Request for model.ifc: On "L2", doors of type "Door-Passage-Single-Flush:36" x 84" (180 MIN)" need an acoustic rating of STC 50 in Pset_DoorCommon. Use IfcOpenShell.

First a look at what the model holds.

```python
import ifcopenshell
import ifcopenshell.util.element

model = ifcopenshell.open("model.ifc")
print(model.schema)
storey = next(s for s in model.by_type("IfcBuildingStorey") if s.Name == "L2")
doors = [e for e in ifcopenshell.util.element.get_decomposition(storey) if e.is_a("IfcDoor")]
seen = {}
for e in doors:
    element_type = ifcopenshell.util.element.get_type(e)
    key = (element_type.Name if element_type != e and element_type else None, ifcopenshell.util.element.get_pset(e, "Pset_DoorCommon", "AcousticRating"))
    seen[key] = seen.get(key, 0) + 1
for (name, value), count in sorted(seen.items(), key=str):
    print(count, "x", name, "|", value)
```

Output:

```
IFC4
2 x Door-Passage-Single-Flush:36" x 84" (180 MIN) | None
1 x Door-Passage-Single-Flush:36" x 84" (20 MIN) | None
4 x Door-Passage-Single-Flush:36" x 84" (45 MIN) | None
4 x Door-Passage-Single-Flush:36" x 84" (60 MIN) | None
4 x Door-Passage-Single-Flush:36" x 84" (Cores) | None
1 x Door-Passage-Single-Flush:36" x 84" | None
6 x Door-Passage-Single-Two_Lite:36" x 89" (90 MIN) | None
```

```python
import ifcopenshell
import ifcopenshell.api.pset
import ifcopenshell.util.element

model = ifcopenshell.open("model.ifc")

storey = next(s for s in model.by_type("IfcBuildingStorey") if s.Name == "L2")
doors = [e for e in ifcopenshell.util.element.get_decomposition(storey) if e.is_a("IfcDoor")]

count = 0
for e in doors:
    element_type = ifcopenshell.util.element.get_type(e)
    if element_type in (None, e) or element_type.Name != 'Door-Passage-Single-Flush:36" x 84" (180 MIN)':
        continue
    # add_pset returns the element's existing set when there is one.
    pset = ifcopenshell.api.pset.add_pset(model, product=e, name="Pset_DoorCommon")
    ifcopenshell.api.pset.edit_pset(model, pset=pset, properties={"AcousticRating": "STC 50"})
    count += 1

print(count, "doors updated")

model.write("model_updated.ifc")
```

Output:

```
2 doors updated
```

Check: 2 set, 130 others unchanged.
